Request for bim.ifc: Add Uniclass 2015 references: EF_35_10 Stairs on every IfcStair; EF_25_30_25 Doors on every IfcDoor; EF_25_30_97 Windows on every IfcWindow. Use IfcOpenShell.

First a look at what the model holds.

```python
import ifcopenshell

model = ifcopenshell.open("bim.ifc")
print(model.schema)
print("classifications:", [c.Name for c in model.by_type("IfcClassification")])
for ifc_class in ("IfcDoor", "IfcRoof", "IfcStair", "IfcWall", "IfcWindow"):
    print(ifc_class, len(model.by_type(ifc_class)))
```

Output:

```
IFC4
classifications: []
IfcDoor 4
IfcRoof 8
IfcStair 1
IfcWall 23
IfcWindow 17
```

```python
import ifcopenshell
import ifcopenshell.api.classification

model = ifcopenshell.open("bim.ifc")

system = ifcopenshell.api.classification.add_classification(model, classification="Uniclass 2015")

codes = {
    "IfcStair": ("EF_35_10", "Stairs"),
    "IfcDoor": ("EF_25_30_25", "Doors"),
    "IfcWindow": ("EF_25_30_97", "Windows"),
}
for ifc_class, (code, name) in codes.items():
    products = model.by_type(ifc_class)
    ifcopenshell.api.classification.add_reference(
        model, products=products, classification=system, identification=code, name=name
    )
    print(code, len(products))

model.write("bim_updated.ifc")
```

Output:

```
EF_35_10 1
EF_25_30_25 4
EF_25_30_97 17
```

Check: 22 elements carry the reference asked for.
